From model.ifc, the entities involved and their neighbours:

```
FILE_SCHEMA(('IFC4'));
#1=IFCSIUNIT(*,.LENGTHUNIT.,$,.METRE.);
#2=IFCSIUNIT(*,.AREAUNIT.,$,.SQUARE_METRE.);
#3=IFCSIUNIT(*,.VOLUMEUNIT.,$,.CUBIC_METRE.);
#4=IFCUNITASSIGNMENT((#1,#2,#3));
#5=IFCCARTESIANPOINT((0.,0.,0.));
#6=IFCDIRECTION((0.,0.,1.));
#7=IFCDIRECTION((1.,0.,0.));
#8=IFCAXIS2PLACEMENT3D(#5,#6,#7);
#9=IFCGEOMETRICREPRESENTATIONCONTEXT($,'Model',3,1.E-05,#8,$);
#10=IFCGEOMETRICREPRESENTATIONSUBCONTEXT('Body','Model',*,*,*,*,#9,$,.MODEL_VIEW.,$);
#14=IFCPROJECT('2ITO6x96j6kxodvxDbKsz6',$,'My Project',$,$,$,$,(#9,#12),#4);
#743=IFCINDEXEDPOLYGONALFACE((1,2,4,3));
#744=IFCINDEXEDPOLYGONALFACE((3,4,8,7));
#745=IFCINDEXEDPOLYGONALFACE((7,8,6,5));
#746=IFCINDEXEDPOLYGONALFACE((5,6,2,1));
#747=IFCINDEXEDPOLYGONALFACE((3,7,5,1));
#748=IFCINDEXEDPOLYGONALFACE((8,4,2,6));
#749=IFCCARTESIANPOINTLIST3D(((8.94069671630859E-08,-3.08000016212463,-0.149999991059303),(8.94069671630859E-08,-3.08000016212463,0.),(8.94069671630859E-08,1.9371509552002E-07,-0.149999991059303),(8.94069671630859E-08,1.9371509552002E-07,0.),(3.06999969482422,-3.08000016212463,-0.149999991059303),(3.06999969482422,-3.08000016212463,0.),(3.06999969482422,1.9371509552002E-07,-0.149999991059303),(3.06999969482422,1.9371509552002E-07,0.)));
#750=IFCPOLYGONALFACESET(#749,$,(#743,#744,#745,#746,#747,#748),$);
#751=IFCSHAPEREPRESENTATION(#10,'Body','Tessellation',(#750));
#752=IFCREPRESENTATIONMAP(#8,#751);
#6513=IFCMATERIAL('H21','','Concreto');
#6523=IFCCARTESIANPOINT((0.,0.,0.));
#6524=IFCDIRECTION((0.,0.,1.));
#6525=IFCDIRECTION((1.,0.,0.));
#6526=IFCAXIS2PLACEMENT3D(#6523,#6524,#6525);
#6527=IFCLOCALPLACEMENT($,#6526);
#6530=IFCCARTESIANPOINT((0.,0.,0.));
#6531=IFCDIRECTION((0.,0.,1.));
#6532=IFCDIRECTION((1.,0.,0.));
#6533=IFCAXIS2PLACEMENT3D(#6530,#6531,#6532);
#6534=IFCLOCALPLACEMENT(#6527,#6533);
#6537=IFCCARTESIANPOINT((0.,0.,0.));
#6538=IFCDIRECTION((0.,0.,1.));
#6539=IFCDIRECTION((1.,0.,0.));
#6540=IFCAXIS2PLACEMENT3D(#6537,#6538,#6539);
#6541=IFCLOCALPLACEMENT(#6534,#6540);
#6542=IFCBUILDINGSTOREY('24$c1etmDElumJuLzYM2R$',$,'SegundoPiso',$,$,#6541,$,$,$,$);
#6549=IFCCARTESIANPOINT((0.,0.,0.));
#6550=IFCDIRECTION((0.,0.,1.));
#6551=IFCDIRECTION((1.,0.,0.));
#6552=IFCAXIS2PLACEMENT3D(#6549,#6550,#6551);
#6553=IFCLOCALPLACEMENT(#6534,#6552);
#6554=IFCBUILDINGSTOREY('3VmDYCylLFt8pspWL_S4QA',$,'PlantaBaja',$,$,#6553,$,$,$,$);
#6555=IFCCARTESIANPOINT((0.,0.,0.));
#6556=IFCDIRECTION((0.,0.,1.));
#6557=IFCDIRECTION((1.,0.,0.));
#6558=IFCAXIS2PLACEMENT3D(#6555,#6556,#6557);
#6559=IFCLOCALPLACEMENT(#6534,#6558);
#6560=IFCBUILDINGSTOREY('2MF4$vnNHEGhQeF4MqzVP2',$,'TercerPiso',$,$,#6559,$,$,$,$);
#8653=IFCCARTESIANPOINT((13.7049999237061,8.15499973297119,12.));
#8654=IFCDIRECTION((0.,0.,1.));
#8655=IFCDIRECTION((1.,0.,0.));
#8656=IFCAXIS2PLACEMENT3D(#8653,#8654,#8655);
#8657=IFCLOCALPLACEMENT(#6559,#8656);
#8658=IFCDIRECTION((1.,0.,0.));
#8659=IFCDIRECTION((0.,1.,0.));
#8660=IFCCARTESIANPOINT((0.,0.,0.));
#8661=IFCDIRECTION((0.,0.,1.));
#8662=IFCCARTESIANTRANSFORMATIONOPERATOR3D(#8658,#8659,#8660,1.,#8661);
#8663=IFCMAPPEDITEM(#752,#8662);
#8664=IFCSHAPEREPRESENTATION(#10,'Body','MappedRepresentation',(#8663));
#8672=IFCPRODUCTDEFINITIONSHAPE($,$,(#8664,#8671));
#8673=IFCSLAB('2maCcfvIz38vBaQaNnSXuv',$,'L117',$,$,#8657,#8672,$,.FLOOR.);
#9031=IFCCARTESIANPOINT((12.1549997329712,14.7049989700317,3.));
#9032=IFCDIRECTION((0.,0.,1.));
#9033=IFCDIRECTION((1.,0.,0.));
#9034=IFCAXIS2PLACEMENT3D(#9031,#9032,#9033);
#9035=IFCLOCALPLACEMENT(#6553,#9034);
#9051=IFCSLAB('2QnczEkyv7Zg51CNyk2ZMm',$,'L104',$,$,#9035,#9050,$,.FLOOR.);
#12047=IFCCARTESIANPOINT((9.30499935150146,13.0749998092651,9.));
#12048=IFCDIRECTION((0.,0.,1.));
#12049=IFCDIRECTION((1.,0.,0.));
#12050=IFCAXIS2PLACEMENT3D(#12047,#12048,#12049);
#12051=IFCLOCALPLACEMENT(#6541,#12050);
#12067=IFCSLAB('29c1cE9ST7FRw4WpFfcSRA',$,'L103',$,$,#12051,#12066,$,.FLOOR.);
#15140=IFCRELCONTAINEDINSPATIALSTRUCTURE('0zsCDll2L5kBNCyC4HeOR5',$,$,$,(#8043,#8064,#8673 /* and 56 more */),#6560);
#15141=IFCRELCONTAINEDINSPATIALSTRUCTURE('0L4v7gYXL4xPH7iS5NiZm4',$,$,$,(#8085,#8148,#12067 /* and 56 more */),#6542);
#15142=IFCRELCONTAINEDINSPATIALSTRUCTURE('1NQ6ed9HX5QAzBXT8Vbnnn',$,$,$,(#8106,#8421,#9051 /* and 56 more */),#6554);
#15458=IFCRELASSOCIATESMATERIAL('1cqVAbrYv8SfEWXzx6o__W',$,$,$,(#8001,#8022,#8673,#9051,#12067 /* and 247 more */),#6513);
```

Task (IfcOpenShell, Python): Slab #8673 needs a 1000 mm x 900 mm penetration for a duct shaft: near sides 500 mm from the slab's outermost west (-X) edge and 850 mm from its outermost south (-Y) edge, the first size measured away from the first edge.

```python
import numpy as np
import ifcopenshell
import ifcopenshell.api.feature
import ifcopenshell.api.geometry
import ifcopenshell.api.root
import ifcopenshell.geom
import ifcopenshell.util.placement
import ifcopenshell.util.representation
import ifcopenshell.util.shape
import ifcopenshell.util.unit

model = ifcopenshell.open("model.ifc")
unit_scale = ifcopenshell.util.unit.calculate_unit_scale(model)
settings = ifcopenshell.geom.settings()


def volume(element):
    """Net volume in cubic metres, openings subtracted."""
    shape = ifcopenshell.geom.create_shape(settings, element)
    return ifcopenshell.util.shape.get_volume(shape.geometry)


slab = model.by_id(8673)
before = volume(slab)

# Extent in the slab's own axes, in metres. The edges named are its -X and -Y sides.
slab_shape = ifcopenshell.geom.create_shape(settings, slab)
vertices = ifcopenshell.util.shape.get_vertices(slab_shape.geometry)
x_min, y_min, bottom = vertices.min(axis=0)
top = vertices[:, 2].max()

opening = ifcopenshell.api.root.create_entity(model, ifc_class="IfcOpeningElement", name="Duct shaft opening", predefined_type="OPENING")
context = ifcopenshell.util.representation.get_context(model, "Model", "Body", "MODEL_VIEW")
width, depth = 1, 0.9
outline = [(0.0, 0.0), (width, 0.0), (width, depth), (0.0, depth), (0.0, 0.0)]
# Overshoot both faces by 50 mm so the cut is clean.
shape = ifcopenshell.api.geometry.add_slab_representation(
    model, context=context, depth=top - bottom + 0.1, polyline=outline
)
ifcopenshell.api.geometry.assign_representation(model, product=opening, representation=shape)

matrix = ifcopenshell.util.placement.get_local_placement(slab.ObjectPlacement)
matrix[:, 3] = matrix @ np.append(np.array([x_min + 0.5, y_min + 0.85, bottom - 0.05]) / unit_scale, 1.0)
ifcopenshell.api.geometry.edit_object_placement(model, product=opening, matrix=matrix, is_si=False)
ifcopenshell.api.feature.add_feature(model, feature=opening, element=slab)

after = volume(slab)

print(f"slab volume {before:.3f} -> {after:.3f} m3")

model.write("model_updated.ifc")
```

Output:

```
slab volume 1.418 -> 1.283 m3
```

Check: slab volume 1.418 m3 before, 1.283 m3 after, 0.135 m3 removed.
